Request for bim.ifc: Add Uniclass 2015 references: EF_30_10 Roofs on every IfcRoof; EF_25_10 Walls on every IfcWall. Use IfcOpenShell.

First a look at what the model holds.

```python
import ifcopenshell

model = ifcopenshell.open("bim.ifc")
print(model.schema)
print("classifications:", [c.Name for c in model.by_type("IfcClassification")])
for ifc_class in ("IfcDoor", "IfcRoof", "IfcStair", "IfcWall", "IfcWindow"):
    print(ifc_class, len(model.by_type(ifc_class)))
```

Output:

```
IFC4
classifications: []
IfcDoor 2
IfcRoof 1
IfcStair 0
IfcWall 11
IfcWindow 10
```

```python
import ifcopenshell
import ifcopenshell.api.classification

model = ifcopenshell.open("bim.ifc")

system = ifcopenshell.api.classification.add_classification(model, classification="Uniclass 2015")

codes = {
    "IfcRoof": ("EF_30_10", "Roofs"),
    "IfcWall": ("EF_25_10", "Walls"),
}
for ifc_class, (code, name) in codes.items():
    products = model.by_type(ifc_class)
    ifcopenshell.api.classification.add_reference(
        model, products=products, classification=system, identification=code, name=name
    )
    print(code, len(products))

model.write("bim-out.ifc")
```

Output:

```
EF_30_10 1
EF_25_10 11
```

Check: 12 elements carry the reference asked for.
